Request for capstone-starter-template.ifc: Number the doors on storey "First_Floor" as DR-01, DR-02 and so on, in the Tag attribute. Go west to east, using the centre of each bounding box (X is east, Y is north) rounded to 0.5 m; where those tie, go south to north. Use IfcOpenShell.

First a look at what the model holds.

```python
import ifcopenshell
import ifcopenshell.util.element
import ifcopenshell.util.placement

model = ifcopenshell.open("capstone-starter-template.ifc")
print(model.schema)
storey = next(s for s in model.by_type("IfcBuildingStorey") if s.Name == "First_Floor")
doors = [e for e in ifcopenshell.util.element.get_decomposition(storey) if e.is_a("IfcDoor")]
for e in sorted(doors, key=lambda e: e.id()):
    origin = ifcopenshell.util.placement.get_local_placement(e.ObjectPlacement)[:3, 3]
    print(e.id(), e.Tag, e.Name, origin.round(2) + 0.0, sep=" | ")
```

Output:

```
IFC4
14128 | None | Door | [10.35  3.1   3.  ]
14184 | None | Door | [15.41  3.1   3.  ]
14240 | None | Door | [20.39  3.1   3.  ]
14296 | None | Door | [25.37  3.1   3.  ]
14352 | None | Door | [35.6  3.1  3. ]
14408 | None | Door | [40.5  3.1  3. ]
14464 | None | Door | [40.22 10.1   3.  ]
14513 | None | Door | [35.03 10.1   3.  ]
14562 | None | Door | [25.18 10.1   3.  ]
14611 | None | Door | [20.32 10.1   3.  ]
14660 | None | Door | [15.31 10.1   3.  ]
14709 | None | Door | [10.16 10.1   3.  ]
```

```python
import ifcopenshell
import ifcopenshell.geom
import ifcopenshell.util.element
import ifcopenshell.util.shape

model = ifcopenshell.open("capstone-starter-template.ifc")
settings = ifcopenshell.geom.settings()
settings.set("use-world-coords", True)


def centre(element):
    shape = ifcopenshell.geom.create_shape(settings, element)
    return ifcopenshell.util.shape.get_bbox_centroid(shape.geometry)


storey = next(s for s in model.by_type("IfcBuildingStorey") if s.Name == "First_Floor")
doors = [e for e in ifcopenshell.util.element.get_decomposition(storey) if e.is_a("IfcDoor")]

# Insertion points can sit at a corner or the storey origin, so sort by the geometry (in metres).
centres = {e: centre(e) for e in doors}
doors.sort(key=lambda e: (round(centres[e][0] / 0.5), centres[e][1]))

for i, e in enumerate(doors, start=1):
    number = f"DR-{i:02d}"
    e.Tag = number
    print(e.id(), number)

model.write("capstone-starter-template_updated.ifc")
```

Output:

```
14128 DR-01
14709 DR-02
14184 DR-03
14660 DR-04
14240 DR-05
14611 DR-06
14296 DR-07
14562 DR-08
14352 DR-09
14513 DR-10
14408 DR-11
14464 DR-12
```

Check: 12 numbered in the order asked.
